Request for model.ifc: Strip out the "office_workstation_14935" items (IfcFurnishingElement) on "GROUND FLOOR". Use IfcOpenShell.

First a look at what the model holds.

```python
import ifcopenshell
import ifcopenshell.util.element

model = ifcopenshell.open("model.ifc")
print(model.schema)
storey = next(s for s in model.by_type("IfcBuildingStorey") if s.Name == "GROUND FLOOR")
furniture = [e for e in ifcopenshell.util.element.get_decomposition(storey) if e.is_a("IfcFurnishingElement")]
seen = {}
for e in furniture:
    element_type = ifcopenshell.util.element.get_type(e)
    name = element_type.Name if element_type not in (None, e) else None
    seen[name] = seen.get(name, 0) + 1
for name, count in sorted(seen.items(), key=str):
    print(count, "x", name)
```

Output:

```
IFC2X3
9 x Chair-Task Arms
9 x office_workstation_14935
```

```python
import ifcopenshell
import ifcopenshell.api.root
import ifcopenshell.util.element

model = ifcopenshell.open("model.ifc")

storey = next(s for s in model.by_type("IfcBuildingStorey") if s.Name == "GROUND FLOOR")
furniture = [e for e in ifcopenshell.util.element.get_decomposition(storey) if e.is_a("IfcFurnishingElement")]
targets = [e for e in furniture if (t := ifcopenshell.util.element.get_type(e)) not in (None, e) and t.Name == "office_workstation_14935"]

for e in targets:
    ifcopenshell.api.root.remove_product(model, product=e)
print(len(targets), "removed")

model.write("model_v2.ifc")
```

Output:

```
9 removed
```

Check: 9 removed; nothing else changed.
